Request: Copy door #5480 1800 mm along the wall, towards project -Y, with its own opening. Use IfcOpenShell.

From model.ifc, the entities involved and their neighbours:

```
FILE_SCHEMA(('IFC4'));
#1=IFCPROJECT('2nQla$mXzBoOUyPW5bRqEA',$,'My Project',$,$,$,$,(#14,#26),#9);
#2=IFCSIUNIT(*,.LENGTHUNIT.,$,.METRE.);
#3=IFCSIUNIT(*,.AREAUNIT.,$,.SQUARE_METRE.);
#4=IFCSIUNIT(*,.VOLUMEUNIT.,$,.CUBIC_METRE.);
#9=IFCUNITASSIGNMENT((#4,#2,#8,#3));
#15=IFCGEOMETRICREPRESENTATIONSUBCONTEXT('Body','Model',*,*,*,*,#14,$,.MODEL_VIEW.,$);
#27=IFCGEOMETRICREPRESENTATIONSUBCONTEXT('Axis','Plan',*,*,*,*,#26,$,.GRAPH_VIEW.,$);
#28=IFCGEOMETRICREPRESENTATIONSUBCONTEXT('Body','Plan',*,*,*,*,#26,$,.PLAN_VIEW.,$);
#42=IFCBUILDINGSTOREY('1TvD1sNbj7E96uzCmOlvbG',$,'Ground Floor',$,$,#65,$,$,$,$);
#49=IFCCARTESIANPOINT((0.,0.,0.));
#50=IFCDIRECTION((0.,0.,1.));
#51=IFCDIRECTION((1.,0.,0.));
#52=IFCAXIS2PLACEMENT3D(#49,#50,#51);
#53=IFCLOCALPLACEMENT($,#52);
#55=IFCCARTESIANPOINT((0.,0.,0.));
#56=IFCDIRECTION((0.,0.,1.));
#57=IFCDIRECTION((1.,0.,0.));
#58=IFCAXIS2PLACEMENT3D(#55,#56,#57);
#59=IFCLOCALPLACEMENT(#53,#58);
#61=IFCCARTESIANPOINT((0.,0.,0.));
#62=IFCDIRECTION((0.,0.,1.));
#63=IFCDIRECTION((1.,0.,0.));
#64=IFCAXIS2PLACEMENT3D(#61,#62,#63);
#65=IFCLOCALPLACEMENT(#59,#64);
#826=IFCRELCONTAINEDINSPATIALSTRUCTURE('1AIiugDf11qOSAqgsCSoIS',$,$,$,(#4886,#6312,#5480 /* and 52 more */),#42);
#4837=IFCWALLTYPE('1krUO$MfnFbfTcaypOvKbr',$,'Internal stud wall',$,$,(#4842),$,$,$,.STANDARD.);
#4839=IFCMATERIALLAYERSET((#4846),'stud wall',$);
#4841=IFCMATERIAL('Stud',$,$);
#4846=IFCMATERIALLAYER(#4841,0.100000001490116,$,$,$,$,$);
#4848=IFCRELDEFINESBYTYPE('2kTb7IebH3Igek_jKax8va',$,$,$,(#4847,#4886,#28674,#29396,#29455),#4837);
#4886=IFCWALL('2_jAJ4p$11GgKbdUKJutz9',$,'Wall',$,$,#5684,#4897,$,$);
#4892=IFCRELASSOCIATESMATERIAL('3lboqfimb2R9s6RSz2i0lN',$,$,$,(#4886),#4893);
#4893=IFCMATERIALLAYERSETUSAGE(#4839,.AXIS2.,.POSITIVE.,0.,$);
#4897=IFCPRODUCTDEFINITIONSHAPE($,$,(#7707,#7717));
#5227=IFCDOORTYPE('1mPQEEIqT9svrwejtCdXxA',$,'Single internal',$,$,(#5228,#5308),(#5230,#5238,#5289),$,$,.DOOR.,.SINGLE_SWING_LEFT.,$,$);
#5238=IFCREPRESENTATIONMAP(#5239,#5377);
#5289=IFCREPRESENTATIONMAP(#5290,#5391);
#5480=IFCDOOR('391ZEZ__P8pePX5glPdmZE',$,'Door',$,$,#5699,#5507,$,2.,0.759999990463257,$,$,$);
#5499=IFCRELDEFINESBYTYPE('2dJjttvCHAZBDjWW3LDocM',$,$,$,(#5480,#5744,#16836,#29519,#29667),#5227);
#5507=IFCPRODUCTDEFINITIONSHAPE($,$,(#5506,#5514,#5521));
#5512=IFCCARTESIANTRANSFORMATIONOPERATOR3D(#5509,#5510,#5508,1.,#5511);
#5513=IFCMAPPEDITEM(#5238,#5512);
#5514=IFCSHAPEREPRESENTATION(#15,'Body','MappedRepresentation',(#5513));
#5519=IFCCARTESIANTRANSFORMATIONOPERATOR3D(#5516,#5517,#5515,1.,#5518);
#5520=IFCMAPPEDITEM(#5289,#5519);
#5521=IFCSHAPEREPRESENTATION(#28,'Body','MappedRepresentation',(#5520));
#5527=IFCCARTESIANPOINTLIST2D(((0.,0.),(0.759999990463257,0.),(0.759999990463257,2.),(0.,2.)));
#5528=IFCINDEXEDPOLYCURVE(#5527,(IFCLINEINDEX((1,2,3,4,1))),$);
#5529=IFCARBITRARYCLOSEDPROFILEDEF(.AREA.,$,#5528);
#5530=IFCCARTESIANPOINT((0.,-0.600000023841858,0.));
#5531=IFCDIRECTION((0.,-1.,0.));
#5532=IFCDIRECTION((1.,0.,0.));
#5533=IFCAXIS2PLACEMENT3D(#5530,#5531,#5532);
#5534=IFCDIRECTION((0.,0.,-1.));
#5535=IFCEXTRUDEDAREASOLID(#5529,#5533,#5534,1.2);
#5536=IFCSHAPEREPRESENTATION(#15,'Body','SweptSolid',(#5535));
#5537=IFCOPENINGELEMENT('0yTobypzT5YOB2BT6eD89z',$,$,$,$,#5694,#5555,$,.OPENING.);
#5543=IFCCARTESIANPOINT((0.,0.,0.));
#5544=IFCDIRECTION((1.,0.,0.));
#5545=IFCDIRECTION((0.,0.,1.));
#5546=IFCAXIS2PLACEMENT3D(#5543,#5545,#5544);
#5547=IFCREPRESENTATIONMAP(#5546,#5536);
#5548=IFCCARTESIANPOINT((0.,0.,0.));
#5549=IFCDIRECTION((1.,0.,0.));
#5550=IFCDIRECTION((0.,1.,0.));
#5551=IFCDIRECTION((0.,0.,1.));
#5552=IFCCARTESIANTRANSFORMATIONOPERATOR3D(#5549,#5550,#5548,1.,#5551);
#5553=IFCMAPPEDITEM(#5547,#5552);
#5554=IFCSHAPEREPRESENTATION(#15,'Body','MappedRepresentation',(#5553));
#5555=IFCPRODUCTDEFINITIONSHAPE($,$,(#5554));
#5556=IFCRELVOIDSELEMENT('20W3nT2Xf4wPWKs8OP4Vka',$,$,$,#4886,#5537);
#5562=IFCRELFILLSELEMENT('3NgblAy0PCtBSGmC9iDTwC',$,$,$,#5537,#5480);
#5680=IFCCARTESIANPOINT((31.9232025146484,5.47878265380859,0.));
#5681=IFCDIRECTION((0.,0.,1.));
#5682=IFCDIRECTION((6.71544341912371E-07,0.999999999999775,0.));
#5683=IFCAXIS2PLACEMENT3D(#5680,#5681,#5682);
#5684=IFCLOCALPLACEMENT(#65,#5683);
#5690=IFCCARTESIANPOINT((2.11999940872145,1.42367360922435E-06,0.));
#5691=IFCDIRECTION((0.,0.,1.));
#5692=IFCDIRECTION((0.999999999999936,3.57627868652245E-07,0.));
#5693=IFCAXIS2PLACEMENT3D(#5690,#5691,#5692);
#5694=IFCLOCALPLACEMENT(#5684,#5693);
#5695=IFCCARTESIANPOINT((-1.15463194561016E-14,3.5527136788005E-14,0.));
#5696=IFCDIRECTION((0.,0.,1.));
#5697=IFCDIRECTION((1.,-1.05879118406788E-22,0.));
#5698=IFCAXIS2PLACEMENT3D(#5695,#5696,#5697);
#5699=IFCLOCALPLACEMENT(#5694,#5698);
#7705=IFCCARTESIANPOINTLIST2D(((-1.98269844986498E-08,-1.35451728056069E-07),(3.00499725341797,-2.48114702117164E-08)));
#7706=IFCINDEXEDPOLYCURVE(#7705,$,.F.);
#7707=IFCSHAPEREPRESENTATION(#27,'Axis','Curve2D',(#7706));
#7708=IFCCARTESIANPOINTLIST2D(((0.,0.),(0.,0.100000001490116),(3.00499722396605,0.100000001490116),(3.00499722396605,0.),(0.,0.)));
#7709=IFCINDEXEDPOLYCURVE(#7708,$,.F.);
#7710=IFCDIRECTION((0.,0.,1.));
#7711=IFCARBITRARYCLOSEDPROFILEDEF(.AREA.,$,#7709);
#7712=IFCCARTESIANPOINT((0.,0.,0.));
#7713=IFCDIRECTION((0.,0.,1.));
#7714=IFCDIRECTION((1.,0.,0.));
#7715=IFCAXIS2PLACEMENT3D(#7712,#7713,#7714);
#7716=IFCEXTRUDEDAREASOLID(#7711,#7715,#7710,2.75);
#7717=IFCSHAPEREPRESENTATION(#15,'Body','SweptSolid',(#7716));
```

```python
import ifcopenshell
import ifcopenshell.api.feature
import ifcopenshell.api.geometry
import ifcopenshell.api.root
import ifcopenshell.geom
import ifcopenshell.util.element
import ifcopenshell.util.placement
import ifcopenshell.util.shape
import ifcopenshell.util.unit

model = ifcopenshell.open("model.ifc")
unit_scale = ifcopenshell.util.unit.calculate_unit_scale(model)
settings = ifcopenshell.geom.settings()


def volume(element):
    """Net volume in cubic metres, openings subtracted."""
    shape = ifcopenshell.geom.create_shape(settings, element)
    return ifcopenshell.util.shape.get_volume(shape.geometry)


door = model.by_guid("391ZEZ__P8pePX5glPdmZE")
opening = door.FillsVoids[0].RelatingOpeningElement
wall = opening.VoidsElements[0].RelatingBuildingElement
before = volume(wall)
shift = ifcopenshell.util.placement.get_local_placement(wall.ObjectPlacement)[:3, 0] * -1.8 / unit_scale

# copy_class copies the void relationship, type, container and properties, but no geometry.
new_opening = ifcopenshell.api.root.copy_class(model, product=opening)
new_opening.Representation = ifcopenshell.util.element.copy_deep(
    model, opening.Representation, exclude=["IfcGeometricRepresentationContext", "IfcRepresentationMap"]
)
new_door = ifcopenshell.api.root.copy_class(model, product=door)
new_door.Representation = ifcopenshell.util.element.copy_deep(
    model, door.Representation, exclude=["IfcGeometricRepresentationContext", "IfcRepresentationMap"]
)
ifcopenshell.api.feature.add_filling(model, opening=new_opening, element=new_door)

for old, new in ((opening, new_opening), (door, new_door)):
    matrix = ifcopenshell.util.placement.get_local_placement(old.ObjectPlacement)
    matrix[:3, 3] += shift
    ifcopenshell.api.geometry.edit_object_placement(model, product=new, matrix=matrix, is_si=False)

after = volume(wall)

print(f"wall volume {before:.3f} -> {after:.3f} m3")

model.write("model_edited.ifc")
```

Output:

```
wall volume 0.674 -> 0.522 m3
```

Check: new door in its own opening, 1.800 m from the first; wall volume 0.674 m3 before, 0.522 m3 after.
